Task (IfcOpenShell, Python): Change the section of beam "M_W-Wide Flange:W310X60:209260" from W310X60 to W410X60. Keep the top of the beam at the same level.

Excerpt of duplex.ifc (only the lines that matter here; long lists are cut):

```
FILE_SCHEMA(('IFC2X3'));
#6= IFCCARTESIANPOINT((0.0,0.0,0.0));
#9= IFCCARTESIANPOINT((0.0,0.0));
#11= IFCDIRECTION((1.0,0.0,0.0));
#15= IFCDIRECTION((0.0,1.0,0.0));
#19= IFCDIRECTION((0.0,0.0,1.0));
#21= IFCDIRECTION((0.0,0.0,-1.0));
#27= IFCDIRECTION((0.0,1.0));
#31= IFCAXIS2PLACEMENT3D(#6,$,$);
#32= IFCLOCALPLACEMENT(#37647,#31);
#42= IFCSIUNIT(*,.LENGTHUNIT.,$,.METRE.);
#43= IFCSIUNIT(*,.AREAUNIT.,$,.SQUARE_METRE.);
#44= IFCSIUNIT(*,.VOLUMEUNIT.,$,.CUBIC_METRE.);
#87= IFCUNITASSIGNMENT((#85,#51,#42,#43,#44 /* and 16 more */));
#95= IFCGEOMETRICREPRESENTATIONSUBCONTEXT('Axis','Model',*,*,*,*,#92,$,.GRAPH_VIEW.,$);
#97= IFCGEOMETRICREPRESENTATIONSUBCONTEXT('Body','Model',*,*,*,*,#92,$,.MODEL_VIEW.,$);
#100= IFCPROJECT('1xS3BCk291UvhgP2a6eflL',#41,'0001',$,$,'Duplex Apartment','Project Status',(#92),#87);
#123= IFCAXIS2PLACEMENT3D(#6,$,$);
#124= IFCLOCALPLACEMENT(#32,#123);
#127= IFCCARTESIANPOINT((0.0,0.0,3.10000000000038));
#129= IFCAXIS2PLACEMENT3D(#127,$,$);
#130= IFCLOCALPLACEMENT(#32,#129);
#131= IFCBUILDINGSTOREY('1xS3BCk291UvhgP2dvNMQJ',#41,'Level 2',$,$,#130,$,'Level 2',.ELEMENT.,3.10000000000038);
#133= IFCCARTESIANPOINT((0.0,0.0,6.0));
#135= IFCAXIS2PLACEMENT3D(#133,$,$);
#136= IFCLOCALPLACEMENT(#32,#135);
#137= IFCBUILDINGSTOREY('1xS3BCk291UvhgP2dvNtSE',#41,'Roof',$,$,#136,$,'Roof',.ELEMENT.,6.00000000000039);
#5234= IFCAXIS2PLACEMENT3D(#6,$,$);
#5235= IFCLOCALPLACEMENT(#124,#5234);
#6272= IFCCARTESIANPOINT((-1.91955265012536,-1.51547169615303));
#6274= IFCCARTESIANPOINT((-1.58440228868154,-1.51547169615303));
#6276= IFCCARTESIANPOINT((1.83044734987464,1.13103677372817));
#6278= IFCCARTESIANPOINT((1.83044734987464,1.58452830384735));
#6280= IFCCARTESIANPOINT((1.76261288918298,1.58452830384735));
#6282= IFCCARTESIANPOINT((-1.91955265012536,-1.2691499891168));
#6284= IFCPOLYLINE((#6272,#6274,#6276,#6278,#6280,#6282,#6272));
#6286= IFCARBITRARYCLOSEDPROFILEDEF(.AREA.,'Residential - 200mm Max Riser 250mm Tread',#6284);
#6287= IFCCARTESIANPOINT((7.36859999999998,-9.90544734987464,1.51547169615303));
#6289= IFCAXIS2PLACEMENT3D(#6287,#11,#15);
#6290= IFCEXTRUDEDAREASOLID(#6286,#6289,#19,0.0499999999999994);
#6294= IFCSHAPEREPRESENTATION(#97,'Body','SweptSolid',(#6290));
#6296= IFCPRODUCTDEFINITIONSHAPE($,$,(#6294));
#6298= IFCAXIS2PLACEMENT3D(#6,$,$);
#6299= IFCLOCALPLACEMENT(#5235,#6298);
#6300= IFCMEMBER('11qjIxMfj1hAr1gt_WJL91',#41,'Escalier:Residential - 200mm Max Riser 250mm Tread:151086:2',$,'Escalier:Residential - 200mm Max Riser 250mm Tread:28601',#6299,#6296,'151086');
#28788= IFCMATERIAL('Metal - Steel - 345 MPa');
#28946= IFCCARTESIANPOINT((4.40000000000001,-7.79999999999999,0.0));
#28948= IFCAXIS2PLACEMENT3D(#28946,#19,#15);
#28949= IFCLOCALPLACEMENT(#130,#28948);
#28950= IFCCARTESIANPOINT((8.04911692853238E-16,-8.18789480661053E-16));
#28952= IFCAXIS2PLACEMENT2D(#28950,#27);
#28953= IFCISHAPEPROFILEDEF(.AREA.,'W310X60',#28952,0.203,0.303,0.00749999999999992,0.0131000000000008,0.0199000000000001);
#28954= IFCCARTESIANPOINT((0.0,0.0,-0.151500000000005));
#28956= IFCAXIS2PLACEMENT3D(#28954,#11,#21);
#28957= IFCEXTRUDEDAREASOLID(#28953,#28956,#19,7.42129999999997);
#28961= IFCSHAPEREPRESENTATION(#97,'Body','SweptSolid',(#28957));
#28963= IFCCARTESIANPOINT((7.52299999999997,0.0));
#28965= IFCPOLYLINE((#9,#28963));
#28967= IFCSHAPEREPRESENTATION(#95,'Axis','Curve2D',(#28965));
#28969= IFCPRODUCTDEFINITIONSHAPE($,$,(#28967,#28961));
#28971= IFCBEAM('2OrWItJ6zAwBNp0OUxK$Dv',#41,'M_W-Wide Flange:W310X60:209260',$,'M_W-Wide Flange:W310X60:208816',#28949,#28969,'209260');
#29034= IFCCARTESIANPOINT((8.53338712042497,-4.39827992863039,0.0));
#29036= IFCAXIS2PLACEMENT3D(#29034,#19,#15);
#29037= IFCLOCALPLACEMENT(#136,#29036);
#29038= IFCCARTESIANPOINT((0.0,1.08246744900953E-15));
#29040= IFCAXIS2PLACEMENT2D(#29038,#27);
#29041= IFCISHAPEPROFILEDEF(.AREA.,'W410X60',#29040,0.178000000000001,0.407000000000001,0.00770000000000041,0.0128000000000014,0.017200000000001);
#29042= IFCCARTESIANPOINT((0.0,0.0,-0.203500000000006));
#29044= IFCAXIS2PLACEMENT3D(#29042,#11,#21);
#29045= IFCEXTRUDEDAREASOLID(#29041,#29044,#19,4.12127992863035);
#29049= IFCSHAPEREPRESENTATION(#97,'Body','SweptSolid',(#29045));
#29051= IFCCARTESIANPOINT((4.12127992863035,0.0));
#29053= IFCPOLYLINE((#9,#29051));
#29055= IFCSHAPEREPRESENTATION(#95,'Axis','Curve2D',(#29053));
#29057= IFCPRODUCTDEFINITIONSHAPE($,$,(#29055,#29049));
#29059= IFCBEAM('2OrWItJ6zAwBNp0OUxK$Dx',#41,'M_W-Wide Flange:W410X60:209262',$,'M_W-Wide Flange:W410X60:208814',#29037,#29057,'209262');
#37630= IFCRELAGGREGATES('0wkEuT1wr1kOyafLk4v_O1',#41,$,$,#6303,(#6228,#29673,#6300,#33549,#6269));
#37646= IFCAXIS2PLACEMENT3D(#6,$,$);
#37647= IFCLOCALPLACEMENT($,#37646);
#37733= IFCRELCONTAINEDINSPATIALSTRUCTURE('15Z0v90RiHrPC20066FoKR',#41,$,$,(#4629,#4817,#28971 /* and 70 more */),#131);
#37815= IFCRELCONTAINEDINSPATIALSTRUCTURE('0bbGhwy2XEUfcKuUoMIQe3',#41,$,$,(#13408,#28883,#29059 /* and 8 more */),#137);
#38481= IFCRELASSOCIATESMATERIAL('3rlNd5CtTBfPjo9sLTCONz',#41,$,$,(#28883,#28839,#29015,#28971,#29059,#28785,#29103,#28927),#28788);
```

```python
import ifcopenshell
import ifcopenshell.util.element
import ifcopenshell.util.representation

model = ifcopenshell.open("duplex.ifc")

member = model.by_guid("2OrWItJ6zAwBNp0OUxK$Dv")
source = next(p for p in model.by_type("IfcIShapeProfileDef") if p.ProfileName == "W410X60")

body = ifcopenshell.util.representation.get_representation(member, "Model", "Body")
solid = body.Items[0]
old_profile = solid.SweptArea

# Copy the section's sizes but keep this member's own profile position.
profile = ifcopenshell.util.element.copy(model, source)
# Profiles are centred, so shift by half the change in depth to hold the top.
shift = (old_profile.OverallDepth - profile.OverallDepth) / 2
x, y = old_profile.Position.Location.Coordinates
up = (-1.0, 0.0)  # upwards, in the solid's own plane
location = model.createIfcCartesianPoint((x + up[0] * shift, y + up[1] * shift))
profile.Position = model.createIfcAxis2Placement2D(location, old_profile.Position.RefDirection)
solid.SweptArea = profile
if not model.get_total_inverses(old_profile):
    ifcopenshell.util.element.remove_deep2(model, old_profile)
member.Name = member.Name.replace("W310X60", "W410X60")
member.ObjectType = member.ObjectType.replace("W310X60", "W410X60")

print(solid.SweptArea)

model.write("duplex_rev.ifc")
```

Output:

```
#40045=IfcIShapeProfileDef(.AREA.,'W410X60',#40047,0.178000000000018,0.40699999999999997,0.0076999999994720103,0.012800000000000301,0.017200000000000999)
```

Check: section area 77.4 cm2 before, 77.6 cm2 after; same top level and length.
